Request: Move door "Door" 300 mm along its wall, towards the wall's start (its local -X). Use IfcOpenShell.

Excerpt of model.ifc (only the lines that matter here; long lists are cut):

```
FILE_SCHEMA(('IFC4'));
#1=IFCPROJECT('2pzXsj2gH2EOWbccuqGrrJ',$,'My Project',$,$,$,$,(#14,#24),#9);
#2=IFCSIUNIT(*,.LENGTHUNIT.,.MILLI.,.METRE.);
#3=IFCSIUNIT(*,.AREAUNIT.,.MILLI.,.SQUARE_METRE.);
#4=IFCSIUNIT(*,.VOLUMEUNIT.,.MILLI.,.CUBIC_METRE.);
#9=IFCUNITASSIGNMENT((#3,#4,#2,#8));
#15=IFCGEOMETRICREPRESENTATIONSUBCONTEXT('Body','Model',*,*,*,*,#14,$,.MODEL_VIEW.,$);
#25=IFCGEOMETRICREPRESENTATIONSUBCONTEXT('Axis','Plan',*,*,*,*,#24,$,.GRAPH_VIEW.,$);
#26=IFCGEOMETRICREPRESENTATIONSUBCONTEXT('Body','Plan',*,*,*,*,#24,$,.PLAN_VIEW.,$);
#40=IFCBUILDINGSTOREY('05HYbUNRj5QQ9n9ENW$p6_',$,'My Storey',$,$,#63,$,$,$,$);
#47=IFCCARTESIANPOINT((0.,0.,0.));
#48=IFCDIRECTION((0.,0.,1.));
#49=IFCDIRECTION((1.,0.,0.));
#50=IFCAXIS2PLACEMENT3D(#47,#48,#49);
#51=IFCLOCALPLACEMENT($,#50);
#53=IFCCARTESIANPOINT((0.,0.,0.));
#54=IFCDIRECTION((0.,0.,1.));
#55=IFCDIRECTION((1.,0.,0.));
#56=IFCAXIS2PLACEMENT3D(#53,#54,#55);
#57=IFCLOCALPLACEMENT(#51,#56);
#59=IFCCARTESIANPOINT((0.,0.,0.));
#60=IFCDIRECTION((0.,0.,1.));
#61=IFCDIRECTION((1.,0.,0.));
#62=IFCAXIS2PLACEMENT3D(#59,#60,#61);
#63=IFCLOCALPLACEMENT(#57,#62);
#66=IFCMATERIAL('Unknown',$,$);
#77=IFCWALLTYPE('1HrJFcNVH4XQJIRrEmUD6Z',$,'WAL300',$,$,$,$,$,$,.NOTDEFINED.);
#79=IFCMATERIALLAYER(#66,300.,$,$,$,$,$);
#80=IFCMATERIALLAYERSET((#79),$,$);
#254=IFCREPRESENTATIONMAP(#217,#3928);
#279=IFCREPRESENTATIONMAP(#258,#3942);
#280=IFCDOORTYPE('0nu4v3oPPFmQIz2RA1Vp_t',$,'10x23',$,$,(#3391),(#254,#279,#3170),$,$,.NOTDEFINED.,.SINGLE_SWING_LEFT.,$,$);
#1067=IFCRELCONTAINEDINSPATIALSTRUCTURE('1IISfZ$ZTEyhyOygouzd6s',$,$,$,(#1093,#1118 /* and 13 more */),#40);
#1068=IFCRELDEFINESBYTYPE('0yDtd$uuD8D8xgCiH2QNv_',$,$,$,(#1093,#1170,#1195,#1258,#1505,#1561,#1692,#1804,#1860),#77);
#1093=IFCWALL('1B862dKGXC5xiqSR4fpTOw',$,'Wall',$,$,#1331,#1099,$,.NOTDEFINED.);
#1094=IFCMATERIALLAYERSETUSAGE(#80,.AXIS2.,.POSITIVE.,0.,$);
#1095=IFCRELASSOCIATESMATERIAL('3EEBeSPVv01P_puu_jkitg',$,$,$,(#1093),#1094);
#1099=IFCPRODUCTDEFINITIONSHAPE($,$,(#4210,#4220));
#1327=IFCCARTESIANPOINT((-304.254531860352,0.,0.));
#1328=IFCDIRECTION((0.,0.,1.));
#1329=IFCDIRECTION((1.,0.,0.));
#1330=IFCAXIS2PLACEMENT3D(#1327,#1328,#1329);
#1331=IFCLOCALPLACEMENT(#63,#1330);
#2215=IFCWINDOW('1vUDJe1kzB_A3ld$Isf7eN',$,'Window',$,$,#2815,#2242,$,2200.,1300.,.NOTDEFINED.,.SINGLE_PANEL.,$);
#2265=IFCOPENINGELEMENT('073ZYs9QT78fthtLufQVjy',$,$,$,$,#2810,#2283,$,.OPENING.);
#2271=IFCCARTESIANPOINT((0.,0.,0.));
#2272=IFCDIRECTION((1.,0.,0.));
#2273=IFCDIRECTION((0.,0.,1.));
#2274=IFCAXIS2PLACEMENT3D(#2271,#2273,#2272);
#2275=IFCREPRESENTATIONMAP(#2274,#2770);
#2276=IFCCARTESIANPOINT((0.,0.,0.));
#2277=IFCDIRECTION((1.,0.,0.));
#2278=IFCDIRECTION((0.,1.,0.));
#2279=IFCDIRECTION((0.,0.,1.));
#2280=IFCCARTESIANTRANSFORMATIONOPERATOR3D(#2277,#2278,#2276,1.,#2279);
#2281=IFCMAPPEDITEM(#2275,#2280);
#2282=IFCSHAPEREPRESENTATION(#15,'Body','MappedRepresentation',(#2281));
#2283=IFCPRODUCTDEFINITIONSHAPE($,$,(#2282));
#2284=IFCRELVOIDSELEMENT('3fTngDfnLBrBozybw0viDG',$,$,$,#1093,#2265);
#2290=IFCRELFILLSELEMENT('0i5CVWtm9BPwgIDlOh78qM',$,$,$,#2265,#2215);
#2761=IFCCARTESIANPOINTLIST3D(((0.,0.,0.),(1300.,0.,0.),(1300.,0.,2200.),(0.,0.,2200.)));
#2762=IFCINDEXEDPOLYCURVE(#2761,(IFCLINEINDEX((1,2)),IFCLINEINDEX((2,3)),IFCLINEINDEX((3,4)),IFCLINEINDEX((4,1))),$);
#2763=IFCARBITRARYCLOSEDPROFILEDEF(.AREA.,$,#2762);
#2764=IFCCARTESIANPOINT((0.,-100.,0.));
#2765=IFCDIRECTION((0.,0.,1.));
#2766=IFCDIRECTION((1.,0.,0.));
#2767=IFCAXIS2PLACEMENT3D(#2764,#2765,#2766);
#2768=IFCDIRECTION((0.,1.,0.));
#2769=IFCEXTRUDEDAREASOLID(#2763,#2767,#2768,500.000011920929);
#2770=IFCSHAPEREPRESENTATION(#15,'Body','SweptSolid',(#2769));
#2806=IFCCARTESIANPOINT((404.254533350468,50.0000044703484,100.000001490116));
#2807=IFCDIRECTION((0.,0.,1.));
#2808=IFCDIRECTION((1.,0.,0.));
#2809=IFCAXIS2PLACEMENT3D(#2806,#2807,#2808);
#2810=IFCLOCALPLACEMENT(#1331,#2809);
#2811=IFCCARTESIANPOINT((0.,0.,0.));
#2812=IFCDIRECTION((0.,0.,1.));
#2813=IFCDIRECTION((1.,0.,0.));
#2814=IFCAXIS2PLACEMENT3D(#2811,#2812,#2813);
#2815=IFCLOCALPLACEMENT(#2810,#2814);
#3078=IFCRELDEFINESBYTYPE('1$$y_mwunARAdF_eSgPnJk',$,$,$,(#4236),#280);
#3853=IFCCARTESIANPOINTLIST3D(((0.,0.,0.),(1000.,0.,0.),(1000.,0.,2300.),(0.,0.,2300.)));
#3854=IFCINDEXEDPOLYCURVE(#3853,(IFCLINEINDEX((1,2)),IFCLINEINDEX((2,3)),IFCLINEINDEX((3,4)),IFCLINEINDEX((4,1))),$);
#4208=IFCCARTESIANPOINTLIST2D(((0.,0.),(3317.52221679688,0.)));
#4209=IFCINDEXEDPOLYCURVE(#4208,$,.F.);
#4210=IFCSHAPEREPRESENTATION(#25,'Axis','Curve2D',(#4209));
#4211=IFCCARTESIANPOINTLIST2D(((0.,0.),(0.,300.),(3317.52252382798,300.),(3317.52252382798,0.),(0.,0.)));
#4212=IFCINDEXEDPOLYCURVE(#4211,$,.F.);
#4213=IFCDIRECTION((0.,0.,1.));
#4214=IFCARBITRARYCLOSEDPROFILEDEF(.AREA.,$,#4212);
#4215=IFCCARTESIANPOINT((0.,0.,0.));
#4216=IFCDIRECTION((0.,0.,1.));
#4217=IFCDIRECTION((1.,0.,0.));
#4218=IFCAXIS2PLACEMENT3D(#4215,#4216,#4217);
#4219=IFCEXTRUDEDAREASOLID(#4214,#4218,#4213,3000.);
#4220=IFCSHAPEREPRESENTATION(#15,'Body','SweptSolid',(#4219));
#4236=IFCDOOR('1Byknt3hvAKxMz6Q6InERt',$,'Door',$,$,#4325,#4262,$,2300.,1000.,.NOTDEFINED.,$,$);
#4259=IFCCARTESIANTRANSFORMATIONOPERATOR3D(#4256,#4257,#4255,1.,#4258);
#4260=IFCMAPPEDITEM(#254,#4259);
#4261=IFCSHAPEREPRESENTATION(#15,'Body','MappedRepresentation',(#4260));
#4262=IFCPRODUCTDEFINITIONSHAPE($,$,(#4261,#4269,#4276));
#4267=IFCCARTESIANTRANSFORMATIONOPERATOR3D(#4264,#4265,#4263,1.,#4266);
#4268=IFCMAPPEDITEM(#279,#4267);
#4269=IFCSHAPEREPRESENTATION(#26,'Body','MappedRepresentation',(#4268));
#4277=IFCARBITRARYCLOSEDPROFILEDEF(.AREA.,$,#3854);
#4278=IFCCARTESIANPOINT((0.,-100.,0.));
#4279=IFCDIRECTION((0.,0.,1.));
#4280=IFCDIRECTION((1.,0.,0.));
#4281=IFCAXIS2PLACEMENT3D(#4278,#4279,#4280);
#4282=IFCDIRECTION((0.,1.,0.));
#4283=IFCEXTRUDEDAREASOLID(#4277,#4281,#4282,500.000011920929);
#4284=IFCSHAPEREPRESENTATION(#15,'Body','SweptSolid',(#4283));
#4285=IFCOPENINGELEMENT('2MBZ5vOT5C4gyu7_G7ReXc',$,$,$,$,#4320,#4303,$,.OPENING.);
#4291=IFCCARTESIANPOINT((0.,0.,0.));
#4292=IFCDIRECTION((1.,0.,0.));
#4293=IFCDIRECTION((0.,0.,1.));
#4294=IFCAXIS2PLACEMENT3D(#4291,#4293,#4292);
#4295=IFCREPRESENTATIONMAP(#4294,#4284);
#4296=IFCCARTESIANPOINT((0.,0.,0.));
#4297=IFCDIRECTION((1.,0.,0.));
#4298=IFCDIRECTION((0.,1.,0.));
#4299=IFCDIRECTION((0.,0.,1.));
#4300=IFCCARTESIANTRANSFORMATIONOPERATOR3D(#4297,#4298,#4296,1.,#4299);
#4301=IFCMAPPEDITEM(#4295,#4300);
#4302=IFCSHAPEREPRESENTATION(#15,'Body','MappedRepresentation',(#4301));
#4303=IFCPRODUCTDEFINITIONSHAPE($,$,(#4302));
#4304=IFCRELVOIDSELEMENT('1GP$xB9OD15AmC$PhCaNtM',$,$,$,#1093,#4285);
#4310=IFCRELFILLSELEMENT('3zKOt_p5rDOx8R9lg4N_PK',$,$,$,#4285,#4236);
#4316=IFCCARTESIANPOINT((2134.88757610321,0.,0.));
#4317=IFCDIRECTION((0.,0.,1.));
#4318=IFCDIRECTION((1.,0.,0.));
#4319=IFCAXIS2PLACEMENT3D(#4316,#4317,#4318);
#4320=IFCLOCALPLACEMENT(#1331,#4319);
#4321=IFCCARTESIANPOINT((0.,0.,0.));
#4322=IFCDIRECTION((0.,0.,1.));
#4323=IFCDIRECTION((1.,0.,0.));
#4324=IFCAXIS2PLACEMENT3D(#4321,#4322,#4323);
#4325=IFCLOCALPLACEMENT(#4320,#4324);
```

```python
import ifcopenshell
import ifcopenshell.api.geometry
import ifcopenshell.util.placement

model = ifcopenshell.open("model.ifc")

door = model.by_guid("1Byknt3hvAKxMz6Q6InERt")
opening = door.FillsVoids[0].RelatingOpeningElement
wall = opening.VoidsElements[0].RelatingBuildingElement

wall_matrix = ifcopenshell.util.placement.get_local_placement(wall.ObjectPlacement)
shift = wall_matrix[:3, 0] * -300.0
before = ifcopenshell.util.placement.get_local_placement(door.ObjectPlacement)[:3, 3].copy()

# The door is placed relative to its opening, so it follows when the opening moves.
matrix = ifcopenshell.util.placement.get_local_placement(opening.ObjectPlacement)
matrix[:3, 3] += shift
ifcopenshell.api.geometry.edit_object_placement(
    model, product=opening, matrix=matrix, is_si=False, should_transform_children=True
)

after = ifcopenshell.util.placement.get_local_placement(door.ObjectPlacement)[:3, 3]
print("door moved by", (after - before).round(3) + 0.0)

model.write("model_v2.ifc")
```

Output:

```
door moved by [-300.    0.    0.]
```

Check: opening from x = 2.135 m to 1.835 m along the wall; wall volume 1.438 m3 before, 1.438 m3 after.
